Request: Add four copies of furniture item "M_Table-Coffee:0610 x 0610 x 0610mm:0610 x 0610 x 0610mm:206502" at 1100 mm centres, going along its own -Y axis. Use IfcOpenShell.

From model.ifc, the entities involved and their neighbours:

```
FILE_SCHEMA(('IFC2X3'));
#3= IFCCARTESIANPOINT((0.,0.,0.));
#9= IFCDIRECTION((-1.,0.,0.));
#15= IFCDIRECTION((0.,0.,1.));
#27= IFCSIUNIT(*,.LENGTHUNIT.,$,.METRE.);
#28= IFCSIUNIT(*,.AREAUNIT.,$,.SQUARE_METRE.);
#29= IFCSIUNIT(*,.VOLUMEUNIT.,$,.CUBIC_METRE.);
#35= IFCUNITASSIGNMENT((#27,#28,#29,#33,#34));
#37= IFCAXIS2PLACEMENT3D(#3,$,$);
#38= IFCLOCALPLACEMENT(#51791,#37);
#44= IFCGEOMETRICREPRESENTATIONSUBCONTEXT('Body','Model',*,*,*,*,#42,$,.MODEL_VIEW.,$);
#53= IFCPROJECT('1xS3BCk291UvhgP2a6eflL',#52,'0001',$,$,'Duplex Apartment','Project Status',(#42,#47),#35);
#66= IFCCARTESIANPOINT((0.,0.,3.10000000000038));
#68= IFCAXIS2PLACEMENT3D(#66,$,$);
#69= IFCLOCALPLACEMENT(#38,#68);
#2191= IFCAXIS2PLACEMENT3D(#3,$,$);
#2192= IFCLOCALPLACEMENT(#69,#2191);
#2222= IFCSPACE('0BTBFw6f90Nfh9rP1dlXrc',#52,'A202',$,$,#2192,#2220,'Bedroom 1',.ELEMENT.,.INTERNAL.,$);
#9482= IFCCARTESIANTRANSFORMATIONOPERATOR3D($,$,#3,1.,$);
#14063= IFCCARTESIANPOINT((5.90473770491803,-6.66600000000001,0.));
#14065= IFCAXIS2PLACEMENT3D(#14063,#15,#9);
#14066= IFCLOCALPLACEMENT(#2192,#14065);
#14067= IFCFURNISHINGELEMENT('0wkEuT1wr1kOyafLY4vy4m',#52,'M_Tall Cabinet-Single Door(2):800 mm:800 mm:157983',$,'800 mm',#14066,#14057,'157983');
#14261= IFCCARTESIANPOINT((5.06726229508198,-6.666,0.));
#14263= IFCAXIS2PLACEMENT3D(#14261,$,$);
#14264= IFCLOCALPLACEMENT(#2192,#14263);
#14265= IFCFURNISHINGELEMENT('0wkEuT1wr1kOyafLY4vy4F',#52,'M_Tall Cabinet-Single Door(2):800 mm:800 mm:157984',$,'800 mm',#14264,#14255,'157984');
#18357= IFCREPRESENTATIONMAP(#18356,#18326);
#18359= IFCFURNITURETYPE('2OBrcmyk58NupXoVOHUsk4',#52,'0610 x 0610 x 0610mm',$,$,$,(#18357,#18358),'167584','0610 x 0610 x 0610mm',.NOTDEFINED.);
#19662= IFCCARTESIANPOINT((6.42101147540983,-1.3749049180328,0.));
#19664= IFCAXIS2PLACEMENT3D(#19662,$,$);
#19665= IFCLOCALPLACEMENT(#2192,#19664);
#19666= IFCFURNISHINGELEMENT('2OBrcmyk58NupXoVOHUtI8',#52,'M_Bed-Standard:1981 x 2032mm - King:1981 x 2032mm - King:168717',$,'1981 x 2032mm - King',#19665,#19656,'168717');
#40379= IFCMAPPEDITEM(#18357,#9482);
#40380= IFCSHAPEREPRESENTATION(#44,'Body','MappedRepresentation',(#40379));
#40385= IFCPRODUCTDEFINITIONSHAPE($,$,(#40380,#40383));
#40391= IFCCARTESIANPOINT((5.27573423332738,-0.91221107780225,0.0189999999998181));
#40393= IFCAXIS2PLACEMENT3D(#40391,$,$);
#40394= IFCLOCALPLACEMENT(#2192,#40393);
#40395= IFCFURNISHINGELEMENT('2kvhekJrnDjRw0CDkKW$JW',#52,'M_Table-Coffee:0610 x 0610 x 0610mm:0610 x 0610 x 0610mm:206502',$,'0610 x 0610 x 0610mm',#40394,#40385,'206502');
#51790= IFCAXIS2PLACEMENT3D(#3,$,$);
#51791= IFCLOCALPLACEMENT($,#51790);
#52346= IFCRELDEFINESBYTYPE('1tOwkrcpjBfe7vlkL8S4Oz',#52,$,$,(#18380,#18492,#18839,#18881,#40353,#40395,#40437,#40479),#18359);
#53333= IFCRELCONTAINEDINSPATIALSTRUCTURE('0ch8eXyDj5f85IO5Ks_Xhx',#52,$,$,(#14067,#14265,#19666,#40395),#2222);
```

```python
import ifcopenshell
import ifcopenshell.api.geometry
import ifcopenshell.api.root
import ifcopenshell.util.element
import ifcopenshell.util.placement

model = ifcopenshell.open("model.ifc")


def reuse_history(source, copy):
    """copy_class also copies each property set's owner history, people and application; keep the originals."""
    for rel in copy.IsDefinedBy:
        if rel.is_a("IfcRelDefinesByProperties") and (history := rel.RelatingPropertyDefinition.OwnerHistory):
            rel.RelatingPropertyDefinition.OwnerHistory = source.OwnerHistory
            ifcopenshell.util.element.remove_deep2(model, history)


source = model.by_guid("2kvhekJrnDjRw0CDkKW$JW")
base = ifcopenshell.util.placement.get_local_placement(source.ObjectPlacement)
step = -base[:3, 1] * 1.1

for i in range(1, 5):
    copy = ifcopenshell.api.root.copy_class(model, product=source)
    copy.Representation = ifcopenshell.util.element.copy_deep(
        model, source.Representation, exclude=["IfcGeometricRepresentationContext", "IfcRepresentationMap"]
    )
    copy.Name = "M_Table-Coffee:0610 x 0610 x 0610mm:0610 x 0610 x 0610mm"
    copy.Tag = None
    reuse_history(source, copy)
    matrix = base.copy()
    matrix[:3, 3] += i * step
    print("added at", matrix[:3, 3].round(3) + 0.0)
    ifcopenshell.api.geometry.edit_object_placement(model, product=copy, matrix=matrix, is_si=False)

model.write("model_updated.ifc")
```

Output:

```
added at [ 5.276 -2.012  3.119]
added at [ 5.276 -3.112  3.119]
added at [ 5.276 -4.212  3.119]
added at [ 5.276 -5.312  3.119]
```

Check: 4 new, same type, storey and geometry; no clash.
